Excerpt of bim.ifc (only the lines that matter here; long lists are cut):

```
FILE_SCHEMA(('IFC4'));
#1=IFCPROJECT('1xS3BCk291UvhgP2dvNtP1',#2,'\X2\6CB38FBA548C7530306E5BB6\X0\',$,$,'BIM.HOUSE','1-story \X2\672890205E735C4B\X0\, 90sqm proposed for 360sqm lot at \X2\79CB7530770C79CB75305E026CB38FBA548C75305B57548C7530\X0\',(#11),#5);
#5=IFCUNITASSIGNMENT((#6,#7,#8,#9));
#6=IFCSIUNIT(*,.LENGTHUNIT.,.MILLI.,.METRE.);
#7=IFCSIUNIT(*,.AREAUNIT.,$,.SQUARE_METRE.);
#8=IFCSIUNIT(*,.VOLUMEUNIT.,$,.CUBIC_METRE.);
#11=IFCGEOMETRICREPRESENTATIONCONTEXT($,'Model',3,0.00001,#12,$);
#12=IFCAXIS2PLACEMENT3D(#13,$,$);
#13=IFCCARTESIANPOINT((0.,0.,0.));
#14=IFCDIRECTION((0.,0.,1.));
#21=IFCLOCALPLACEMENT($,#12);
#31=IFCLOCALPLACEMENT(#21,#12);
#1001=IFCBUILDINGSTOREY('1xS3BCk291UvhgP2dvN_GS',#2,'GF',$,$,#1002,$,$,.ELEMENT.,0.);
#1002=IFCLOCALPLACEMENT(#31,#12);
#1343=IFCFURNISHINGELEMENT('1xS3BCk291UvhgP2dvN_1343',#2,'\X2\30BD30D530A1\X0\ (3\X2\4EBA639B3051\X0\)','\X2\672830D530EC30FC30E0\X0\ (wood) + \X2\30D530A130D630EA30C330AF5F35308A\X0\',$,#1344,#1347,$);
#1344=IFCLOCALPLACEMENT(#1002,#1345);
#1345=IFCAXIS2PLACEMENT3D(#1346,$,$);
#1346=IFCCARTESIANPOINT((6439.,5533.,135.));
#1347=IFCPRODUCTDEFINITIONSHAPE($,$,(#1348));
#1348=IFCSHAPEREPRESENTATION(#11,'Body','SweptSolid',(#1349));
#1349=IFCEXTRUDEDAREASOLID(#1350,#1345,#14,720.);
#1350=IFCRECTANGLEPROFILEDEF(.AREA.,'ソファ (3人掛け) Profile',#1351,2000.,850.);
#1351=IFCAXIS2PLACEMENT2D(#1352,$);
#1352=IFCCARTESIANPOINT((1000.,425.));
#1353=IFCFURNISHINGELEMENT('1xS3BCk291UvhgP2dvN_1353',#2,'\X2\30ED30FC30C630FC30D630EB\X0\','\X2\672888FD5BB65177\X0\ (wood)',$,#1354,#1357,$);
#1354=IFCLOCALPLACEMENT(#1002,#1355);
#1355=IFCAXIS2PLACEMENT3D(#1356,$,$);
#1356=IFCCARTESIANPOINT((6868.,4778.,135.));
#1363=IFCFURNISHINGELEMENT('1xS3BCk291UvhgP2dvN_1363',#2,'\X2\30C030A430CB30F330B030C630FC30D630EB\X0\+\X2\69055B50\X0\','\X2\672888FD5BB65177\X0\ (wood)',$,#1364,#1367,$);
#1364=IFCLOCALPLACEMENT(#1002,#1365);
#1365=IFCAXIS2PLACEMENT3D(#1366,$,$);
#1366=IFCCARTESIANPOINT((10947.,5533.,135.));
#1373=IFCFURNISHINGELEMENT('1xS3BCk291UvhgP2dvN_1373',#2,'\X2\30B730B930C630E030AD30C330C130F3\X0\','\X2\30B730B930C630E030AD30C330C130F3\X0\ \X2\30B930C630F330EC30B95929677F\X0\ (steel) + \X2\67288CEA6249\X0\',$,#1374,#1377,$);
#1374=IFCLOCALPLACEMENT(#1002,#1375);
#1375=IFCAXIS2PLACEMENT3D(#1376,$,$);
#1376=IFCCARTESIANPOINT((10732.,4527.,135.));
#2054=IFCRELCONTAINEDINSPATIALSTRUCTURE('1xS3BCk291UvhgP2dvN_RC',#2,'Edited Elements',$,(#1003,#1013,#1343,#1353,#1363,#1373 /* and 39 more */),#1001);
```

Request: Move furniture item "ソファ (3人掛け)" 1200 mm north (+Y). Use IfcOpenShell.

```python
import ifcopenshell
import ifcopenshell.api.geometry
import ifcopenshell.util.placement
import ifcopenshell.util.unit

model = ifcopenshell.open("bim.ifc")
unit_scale = ifcopenshell.util.unit.calculate_unit_scale(model)

item = model.by_guid("1xS3BCk291UvhgP2dvN_1343")
matrix = ifcopenshell.util.placement.get_local_placement(item.ObjectPlacement)
matrix[1, 3] += 1.2 / unit_scale
ifcopenshell.api.geometry.edit_object_placement(model, product=item, matrix=matrix, is_si=False)

print(ifcopenshell.util.placement.get_local_placement(item.ObjectPlacement).round(3) + 0.0)

model.write("bim_rev.ifc")
```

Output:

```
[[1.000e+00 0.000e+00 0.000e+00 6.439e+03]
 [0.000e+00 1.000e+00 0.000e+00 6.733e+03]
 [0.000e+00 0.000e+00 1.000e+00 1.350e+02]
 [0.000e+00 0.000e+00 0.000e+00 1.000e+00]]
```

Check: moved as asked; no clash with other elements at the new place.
